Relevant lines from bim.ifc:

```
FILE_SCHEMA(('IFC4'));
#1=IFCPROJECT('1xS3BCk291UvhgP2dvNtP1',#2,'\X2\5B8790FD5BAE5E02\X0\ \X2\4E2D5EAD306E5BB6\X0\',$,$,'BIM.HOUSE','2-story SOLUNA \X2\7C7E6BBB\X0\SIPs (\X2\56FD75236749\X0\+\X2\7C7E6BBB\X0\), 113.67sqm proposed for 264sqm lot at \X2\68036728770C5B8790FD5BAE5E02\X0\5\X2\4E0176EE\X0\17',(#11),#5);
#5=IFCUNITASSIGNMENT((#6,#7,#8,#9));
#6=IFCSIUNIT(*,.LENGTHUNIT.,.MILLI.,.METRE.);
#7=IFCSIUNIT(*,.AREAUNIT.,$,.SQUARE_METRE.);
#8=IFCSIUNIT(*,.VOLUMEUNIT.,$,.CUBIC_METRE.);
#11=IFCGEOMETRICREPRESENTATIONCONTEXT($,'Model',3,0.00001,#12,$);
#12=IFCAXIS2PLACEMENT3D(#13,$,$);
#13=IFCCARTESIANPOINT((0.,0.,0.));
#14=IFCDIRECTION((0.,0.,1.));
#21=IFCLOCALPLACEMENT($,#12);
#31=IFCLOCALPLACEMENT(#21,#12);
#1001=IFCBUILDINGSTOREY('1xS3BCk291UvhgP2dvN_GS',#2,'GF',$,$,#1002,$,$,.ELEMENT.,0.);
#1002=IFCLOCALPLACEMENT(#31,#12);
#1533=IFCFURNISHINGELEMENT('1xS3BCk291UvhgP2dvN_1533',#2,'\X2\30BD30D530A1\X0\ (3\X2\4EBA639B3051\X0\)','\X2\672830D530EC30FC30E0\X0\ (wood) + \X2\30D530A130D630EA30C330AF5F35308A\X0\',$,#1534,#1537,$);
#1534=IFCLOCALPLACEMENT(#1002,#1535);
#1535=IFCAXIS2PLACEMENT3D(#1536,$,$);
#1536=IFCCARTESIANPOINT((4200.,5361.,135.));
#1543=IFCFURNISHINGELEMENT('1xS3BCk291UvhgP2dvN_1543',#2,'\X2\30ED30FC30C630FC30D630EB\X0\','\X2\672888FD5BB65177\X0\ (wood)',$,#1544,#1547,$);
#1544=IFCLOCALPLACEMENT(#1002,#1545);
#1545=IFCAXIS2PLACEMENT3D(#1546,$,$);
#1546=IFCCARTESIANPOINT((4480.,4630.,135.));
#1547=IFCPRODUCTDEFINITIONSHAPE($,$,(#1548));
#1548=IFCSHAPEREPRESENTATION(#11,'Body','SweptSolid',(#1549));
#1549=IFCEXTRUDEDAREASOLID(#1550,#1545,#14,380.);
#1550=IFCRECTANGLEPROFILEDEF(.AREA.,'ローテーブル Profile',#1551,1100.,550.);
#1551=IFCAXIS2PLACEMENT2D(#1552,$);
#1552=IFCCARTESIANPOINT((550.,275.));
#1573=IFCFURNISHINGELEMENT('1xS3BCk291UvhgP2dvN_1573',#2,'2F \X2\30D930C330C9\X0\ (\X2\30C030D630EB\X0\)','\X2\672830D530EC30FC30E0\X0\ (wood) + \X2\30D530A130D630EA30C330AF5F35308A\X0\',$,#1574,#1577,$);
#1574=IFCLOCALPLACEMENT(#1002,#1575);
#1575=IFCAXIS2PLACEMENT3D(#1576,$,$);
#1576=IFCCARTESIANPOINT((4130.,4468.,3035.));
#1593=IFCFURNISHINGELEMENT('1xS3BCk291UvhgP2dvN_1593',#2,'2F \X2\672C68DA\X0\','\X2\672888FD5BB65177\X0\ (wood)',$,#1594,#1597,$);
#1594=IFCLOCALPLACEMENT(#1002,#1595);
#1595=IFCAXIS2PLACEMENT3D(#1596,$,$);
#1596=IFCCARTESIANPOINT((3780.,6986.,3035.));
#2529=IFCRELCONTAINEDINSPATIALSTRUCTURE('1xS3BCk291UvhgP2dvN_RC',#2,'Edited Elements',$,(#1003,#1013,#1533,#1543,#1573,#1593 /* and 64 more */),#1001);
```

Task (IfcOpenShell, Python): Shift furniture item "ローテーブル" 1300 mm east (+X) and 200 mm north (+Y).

```python
import ifcopenshell
import ifcopenshell.api.geometry
import ifcopenshell.util.placement
import ifcopenshell.util.unit

model = ifcopenshell.open("bim.ifc")
unit_scale = ifcopenshell.util.unit.calculate_unit_scale(model)

item = model.by_guid("1xS3BCk291UvhgP2dvN_1543")
matrix = ifcopenshell.util.placement.get_local_placement(item.ObjectPlacement)
matrix[0, 3] += 1.3 / unit_scale
matrix[1, 3] += 0.2 / unit_scale
ifcopenshell.api.geometry.edit_object_placement(model, product=item, matrix=matrix, is_si=False)

print(ifcopenshell.util.placement.get_local_placement(item.ObjectPlacement).round(3) + 0.0)

model.write("bim_updated.ifc")
```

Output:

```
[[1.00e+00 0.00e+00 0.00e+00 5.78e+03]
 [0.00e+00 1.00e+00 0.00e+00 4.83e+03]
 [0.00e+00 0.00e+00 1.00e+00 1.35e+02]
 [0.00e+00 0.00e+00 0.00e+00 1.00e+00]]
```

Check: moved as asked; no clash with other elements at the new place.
